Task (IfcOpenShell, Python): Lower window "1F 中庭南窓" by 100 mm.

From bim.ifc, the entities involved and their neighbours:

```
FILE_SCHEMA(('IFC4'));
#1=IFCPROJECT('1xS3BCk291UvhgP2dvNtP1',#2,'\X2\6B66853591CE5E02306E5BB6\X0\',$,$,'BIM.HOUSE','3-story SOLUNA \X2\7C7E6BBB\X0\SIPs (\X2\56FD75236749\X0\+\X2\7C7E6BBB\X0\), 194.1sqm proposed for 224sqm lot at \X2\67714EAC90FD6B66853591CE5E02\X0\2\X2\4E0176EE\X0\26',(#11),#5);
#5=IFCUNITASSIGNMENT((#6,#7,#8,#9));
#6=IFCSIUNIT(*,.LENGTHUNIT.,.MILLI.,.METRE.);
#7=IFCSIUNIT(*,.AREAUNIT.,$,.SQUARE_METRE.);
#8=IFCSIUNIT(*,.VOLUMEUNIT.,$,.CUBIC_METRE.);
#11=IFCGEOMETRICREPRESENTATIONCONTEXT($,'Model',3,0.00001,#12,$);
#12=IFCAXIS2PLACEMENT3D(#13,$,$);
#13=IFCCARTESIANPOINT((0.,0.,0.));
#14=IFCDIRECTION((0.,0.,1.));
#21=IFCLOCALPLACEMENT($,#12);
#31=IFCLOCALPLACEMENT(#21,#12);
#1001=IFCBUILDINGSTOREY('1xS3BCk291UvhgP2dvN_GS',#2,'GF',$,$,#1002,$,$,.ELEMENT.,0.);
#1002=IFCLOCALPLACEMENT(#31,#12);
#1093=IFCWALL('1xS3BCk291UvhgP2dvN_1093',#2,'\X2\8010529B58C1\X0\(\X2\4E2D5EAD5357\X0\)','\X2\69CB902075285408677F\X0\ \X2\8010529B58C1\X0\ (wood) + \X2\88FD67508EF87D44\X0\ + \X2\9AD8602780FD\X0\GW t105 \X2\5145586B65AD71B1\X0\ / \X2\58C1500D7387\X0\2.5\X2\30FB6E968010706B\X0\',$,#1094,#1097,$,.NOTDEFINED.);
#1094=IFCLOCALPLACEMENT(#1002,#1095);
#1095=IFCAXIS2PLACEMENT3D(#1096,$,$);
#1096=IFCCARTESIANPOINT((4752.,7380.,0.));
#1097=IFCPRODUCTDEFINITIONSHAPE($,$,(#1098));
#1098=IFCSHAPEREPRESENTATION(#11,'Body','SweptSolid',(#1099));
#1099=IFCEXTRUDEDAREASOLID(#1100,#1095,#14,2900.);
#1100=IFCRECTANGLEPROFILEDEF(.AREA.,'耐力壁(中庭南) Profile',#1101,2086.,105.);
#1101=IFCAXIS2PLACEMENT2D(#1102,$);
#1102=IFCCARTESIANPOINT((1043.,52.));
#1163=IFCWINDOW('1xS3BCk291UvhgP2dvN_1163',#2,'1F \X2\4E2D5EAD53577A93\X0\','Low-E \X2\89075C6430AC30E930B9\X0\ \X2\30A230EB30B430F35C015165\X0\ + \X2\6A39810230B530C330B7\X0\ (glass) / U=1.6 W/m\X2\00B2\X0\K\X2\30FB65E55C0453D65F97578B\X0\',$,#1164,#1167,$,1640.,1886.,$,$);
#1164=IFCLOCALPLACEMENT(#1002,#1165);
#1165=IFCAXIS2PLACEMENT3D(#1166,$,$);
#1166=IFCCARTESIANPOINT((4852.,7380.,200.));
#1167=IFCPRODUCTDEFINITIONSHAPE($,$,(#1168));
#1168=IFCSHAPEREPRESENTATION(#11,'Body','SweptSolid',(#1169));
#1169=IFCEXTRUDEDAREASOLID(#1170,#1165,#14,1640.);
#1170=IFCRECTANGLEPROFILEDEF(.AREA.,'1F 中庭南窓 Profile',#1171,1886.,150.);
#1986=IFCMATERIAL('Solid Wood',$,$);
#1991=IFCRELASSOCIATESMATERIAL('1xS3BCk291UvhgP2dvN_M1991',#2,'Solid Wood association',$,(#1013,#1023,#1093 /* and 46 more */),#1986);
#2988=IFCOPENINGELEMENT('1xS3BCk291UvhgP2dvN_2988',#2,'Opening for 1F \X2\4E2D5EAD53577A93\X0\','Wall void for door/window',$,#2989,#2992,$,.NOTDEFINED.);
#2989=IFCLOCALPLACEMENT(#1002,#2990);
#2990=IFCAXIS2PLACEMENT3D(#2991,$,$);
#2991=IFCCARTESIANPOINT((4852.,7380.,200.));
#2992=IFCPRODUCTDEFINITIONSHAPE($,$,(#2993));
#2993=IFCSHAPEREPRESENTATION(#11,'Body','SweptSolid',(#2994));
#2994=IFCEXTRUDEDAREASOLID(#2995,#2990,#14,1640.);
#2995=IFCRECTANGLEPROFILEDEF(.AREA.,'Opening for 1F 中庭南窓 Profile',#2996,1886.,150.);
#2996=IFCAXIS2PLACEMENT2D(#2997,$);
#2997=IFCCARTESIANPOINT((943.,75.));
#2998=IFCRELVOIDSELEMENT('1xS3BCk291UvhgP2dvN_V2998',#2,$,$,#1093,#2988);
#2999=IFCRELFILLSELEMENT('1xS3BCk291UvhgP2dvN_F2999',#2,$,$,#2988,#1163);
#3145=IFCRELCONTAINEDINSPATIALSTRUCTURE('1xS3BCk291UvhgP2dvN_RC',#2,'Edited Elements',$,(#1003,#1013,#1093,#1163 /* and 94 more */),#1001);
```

```python
import numpy as np
import ifcopenshell
import ifcopenshell.api.geometry
import ifcopenshell.util.placement
import ifcopenshell.util.unit

model = ifcopenshell.open("bim.ifc")
unit_scale = ifcopenshell.util.unit.calculate_unit_scale(model)

window = model.by_id(1163)
opening = window.FillsVoids[0].RelatingOpeningElement
dz = -0.1 / unit_scale

shift = np.array([0.0, 0.0, dz])
# The window is not placed relative to its opening, so move both.
for product in (opening, window):
    matrix = ifcopenshell.util.placement.get_local_placement(product.ObjectPlacement)
    matrix[:3, 3] += shift
    ifcopenshell.api.geometry.edit_object_placement(model, product=product, matrix=matrix, is_si=False)

print(f"moved by {dz * unit_scale:+.3f} m")

model.write("bim_rev.ifc")
```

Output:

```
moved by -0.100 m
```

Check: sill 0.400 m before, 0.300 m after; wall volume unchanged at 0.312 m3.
